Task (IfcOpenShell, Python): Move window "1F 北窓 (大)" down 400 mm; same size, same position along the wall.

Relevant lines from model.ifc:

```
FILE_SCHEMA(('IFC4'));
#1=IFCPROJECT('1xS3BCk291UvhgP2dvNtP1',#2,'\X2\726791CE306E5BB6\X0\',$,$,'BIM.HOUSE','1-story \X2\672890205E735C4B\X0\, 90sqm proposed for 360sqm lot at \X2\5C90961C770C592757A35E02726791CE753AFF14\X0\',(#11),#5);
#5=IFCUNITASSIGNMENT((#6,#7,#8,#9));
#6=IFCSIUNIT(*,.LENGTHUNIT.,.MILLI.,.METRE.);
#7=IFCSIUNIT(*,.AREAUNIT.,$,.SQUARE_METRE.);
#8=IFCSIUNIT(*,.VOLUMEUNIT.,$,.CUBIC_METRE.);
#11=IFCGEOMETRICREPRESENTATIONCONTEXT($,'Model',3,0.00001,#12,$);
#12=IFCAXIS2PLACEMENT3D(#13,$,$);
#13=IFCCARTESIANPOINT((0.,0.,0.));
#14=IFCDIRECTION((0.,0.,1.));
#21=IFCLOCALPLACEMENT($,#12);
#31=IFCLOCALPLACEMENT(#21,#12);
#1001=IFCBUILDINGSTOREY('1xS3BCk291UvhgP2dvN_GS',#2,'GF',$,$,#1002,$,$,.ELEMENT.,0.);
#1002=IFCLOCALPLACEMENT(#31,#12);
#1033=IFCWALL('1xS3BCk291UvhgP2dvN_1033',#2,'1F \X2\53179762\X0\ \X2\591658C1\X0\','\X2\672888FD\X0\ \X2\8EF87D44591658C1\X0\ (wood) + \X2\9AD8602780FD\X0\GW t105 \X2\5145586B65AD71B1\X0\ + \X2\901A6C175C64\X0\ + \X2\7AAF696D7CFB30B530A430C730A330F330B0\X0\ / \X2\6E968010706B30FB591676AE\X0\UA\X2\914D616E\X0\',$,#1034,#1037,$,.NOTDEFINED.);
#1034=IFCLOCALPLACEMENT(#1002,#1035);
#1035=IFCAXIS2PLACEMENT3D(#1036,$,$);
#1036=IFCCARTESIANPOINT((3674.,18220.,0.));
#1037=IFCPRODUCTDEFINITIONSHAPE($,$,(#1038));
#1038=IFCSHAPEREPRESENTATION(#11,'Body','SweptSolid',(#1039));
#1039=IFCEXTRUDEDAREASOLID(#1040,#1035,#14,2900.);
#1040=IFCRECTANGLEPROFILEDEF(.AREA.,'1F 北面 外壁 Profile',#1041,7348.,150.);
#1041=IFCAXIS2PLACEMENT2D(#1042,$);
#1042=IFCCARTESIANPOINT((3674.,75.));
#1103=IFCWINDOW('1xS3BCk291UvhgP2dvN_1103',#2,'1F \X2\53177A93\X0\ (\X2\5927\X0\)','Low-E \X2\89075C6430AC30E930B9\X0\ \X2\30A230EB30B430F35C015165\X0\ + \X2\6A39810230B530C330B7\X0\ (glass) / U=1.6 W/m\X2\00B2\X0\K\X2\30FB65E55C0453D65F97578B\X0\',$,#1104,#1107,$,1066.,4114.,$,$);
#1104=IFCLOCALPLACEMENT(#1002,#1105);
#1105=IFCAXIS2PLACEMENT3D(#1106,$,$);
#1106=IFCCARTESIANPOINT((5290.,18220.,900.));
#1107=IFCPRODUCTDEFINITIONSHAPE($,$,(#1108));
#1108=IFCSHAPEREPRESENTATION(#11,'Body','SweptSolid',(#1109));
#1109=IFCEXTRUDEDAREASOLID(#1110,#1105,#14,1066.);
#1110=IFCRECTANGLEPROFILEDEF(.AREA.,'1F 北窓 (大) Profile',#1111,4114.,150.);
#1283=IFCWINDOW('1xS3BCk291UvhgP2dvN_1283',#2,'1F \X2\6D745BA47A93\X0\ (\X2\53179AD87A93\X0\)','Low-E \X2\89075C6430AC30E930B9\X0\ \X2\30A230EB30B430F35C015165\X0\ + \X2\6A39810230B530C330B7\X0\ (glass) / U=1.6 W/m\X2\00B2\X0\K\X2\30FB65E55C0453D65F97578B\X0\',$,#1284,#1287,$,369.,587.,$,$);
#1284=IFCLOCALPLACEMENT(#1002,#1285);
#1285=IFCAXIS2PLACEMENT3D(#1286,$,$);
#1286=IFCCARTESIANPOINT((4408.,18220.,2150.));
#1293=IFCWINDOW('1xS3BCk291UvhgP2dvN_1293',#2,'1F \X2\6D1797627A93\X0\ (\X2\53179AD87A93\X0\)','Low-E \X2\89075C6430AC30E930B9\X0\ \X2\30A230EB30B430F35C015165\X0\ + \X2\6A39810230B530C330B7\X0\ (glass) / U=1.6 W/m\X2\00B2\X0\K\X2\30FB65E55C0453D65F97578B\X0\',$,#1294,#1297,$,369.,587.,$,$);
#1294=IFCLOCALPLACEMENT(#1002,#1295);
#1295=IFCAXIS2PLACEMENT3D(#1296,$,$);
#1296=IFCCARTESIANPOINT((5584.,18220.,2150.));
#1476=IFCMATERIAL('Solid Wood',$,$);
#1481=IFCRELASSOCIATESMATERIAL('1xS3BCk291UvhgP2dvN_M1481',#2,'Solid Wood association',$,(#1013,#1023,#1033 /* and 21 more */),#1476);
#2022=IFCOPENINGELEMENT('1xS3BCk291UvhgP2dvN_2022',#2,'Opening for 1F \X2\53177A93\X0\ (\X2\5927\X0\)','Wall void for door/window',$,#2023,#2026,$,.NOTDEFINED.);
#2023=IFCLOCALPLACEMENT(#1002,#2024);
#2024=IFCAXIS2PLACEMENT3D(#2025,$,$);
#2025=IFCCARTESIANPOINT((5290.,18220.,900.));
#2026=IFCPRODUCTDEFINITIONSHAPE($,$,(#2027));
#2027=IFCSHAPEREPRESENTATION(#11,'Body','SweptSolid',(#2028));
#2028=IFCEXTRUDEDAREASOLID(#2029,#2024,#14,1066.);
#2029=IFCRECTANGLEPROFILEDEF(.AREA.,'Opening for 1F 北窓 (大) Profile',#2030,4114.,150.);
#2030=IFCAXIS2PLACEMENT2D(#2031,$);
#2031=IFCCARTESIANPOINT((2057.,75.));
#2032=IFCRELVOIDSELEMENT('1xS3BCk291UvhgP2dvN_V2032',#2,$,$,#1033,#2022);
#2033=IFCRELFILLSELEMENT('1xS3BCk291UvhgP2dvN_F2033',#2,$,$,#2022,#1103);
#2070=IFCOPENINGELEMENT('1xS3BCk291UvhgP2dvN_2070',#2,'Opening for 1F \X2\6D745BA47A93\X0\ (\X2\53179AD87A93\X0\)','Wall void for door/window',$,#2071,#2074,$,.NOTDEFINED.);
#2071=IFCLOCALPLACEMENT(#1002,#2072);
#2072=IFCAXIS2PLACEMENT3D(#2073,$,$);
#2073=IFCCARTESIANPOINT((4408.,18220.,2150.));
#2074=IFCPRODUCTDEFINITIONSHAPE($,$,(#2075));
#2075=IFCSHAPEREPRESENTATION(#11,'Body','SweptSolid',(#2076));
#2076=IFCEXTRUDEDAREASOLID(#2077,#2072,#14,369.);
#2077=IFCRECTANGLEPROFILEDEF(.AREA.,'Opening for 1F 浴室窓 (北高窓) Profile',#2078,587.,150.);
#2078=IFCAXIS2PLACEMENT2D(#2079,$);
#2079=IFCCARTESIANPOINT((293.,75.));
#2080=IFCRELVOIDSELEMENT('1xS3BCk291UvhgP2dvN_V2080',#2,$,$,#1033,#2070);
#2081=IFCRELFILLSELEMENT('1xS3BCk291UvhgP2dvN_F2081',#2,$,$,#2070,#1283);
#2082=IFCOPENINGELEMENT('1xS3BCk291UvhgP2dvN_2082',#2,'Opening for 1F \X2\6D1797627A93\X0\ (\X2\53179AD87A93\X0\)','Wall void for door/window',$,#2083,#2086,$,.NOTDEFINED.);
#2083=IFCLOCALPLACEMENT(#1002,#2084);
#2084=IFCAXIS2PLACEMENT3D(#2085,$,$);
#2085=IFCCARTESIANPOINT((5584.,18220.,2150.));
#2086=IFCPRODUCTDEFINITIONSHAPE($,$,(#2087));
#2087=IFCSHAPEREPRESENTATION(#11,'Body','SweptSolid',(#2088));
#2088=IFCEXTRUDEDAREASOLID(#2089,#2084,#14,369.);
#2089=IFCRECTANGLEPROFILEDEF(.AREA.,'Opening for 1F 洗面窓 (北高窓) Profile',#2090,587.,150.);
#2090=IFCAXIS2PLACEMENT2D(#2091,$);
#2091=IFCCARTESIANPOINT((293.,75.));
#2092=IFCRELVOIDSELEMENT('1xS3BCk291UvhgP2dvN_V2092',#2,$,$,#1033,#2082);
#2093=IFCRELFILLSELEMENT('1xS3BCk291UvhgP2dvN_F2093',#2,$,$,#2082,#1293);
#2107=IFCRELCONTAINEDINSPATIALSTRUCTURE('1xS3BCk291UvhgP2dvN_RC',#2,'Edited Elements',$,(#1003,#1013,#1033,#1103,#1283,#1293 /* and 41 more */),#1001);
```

```python
import numpy as np
import ifcopenshell
import ifcopenshell.api.geometry
import ifcopenshell.util.placement
import ifcopenshell.util.unit

model = ifcopenshell.open("model.ifc")
unit_scale = ifcopenshell.util.unit.calculate_unit_scale(model)

window = model.by_id(1103)
opening = window.FillsVoids[0].RelatingOpeningElement
dz = -0.4 / unit_scale

shift = np.array([0.0, 0.0, dz])
# The window is not placed relative to its opening, so move both.
for product in (opening, window):
    matrix = ifcopenshell.util.placement.get_local_placement(product.ObjectPlacement)
    matrix[:3, 3] += shift
    ifcopenshell.api.geometry.edit_object_placement(model, product=product, matrix=matrix, is_si=False)

print(f"moved by {dz * unit_scale:+.3f} m")

model.write("model_edited.ifc")
```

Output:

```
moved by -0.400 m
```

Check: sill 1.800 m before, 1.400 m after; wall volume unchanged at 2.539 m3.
